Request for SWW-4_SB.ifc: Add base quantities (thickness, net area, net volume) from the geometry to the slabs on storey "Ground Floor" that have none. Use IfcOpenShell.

First a look at what the model holds.

```python
import ifcopenshell
import ifcopenshell.util.element
import ifcopenshell.util.unit

model = ifcopenshell.open("SWW-4_SB.ifc")
print(model.schema)
for unit_type in ("LENGTHUNIT", "AREAUNIT", "VOLUMEUNIT"):
    print(unit_type, ifcopenshell.util.unit.calculate_unit_scale(model, unit_type))
storey = next(s for s in model.by_type("IfcBuildingStorey") if s.Name == "Ground Floor")
slabs = [e for e in ifcopenshell.util.element.get_decomposition(storey) if e.is_a("IfcSlab")]
for e in sorted(slabs, key=lambda e: e.id()):
    print(e.id(), e.is_a(), e.Name, list(ifcopenshell.util.element.get_psets(e, qtos_only=True)), sep=" | ")
```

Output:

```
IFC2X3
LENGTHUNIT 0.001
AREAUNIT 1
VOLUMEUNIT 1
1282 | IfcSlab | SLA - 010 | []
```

```python
import ifcopenshell
import ifcopenshell.api.pset
import ifcopenshell.geom
import ifcopenshell.util.element
import ifcopenshell.util.shape
import ifcopenshell.util.unit

model = ifcopenshell.open("SWW-4_SB.ifc")
unit_scale = ifcopenshell.util.unit.calculate_unit_scale(model)
area_scale = ifcopenshell.util.unit.calculate_unit_scale(model, "AREAUNIT")
volume_scale = ifcopenshell.util.unit.calculate_unit_scale(model, "VOLUMEUNIT")
settings = ifcopenshell.geom.settings()

storey = next(s for s in model.by_type("IfcBuildingStorey") if s.Name == "Ground Floor")
slabs = [e for e in ifcopenshell.util.element.get_decomposition(storey) if e.is_a("IfcSlab")]

for e in sorted(slabs, key=lambda e: e.id()):
    if ifcopenshell.util.element.get_psets(e, qtos_only=True, should_inherit=False):
        continue
    # Geometry comes back in metres, in the element's own axes.
    shape = ifcopenshell.geom.create_shape(settings, e)
    values = {
        "Width": ifcopenshell.util.shape.get_z(shape.geometry) / unit_scale,
        "NetArea": ifcopenshell.util.shape.get_footprint_area(shape.geometry) / area_scale,
        "NetVolume": ifcopenshell.util.shape.get_volume(shape.geometry) / volume_scale,
    }
    qto = ifcopenshell.api.pset.add_qto(model, product=e, name="BaseQuantities")
    ifcopenshell.api.pset.edit_qto(model, qto=qto, properties=values)
    print(e.id(), {k: round(v, 3) for k, v in values.items()})

model.write("SWW-4_SB_rev.ifc")
```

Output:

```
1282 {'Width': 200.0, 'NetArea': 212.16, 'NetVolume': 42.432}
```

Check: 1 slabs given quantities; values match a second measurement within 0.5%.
